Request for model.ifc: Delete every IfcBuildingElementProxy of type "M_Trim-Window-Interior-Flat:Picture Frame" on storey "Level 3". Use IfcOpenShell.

First a look at what the model holds.

```python
import ifcopenshell
import ifcopenshell.util.element

model = ifcopenshell.open("model.ifc")
print(model.schema)
storey = next(s for s in model.by_type("IfcBuildingStorey") if s.Name == "Level 3")
proxies = [e for e in ifcopenshell.util.element.get_decomposition(storey) if e.is_a("IfcBuildingElementProxy")]
seen = {}
for e in proxies:
    element_type = ifcopenshell.util.element.get_type(e)
    name = element_type.Name if element_type not in (None, e) else None
    seen[name] = seen.get(name, 0) + 1
for name, count in sorted(seen.items(), key=str):
    print(count, "x", name)
```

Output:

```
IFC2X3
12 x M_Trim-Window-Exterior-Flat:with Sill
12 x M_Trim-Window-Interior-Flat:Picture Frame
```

```python
import ifcopenshell
import ifcopenshell.api.root
import ifcopenshell.util.element

model = ifcopenshell.open("model.ifc")

storey = next(s for s in model.by_type("IfcBuildingStorey") if s.Name == "Level 3")
proxies = [e for e in ifcopenshell.util.element.get_decomposition(storey) if e.is_a("IfcBuildingElementProxy")]
targets = [e for e in proxies if (t := ifcopenshell.util.element.get_type(e)) not in (None, e) and t.Name == "M_Trim-Window-Interior-Flat:Picture Frame"]

for e in targets:
    ifcopenshell.api.root.remove_product(model, product=e)
print(len(targets), "removed")

model.write("model_rev.ifc")
```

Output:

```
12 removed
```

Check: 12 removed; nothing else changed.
